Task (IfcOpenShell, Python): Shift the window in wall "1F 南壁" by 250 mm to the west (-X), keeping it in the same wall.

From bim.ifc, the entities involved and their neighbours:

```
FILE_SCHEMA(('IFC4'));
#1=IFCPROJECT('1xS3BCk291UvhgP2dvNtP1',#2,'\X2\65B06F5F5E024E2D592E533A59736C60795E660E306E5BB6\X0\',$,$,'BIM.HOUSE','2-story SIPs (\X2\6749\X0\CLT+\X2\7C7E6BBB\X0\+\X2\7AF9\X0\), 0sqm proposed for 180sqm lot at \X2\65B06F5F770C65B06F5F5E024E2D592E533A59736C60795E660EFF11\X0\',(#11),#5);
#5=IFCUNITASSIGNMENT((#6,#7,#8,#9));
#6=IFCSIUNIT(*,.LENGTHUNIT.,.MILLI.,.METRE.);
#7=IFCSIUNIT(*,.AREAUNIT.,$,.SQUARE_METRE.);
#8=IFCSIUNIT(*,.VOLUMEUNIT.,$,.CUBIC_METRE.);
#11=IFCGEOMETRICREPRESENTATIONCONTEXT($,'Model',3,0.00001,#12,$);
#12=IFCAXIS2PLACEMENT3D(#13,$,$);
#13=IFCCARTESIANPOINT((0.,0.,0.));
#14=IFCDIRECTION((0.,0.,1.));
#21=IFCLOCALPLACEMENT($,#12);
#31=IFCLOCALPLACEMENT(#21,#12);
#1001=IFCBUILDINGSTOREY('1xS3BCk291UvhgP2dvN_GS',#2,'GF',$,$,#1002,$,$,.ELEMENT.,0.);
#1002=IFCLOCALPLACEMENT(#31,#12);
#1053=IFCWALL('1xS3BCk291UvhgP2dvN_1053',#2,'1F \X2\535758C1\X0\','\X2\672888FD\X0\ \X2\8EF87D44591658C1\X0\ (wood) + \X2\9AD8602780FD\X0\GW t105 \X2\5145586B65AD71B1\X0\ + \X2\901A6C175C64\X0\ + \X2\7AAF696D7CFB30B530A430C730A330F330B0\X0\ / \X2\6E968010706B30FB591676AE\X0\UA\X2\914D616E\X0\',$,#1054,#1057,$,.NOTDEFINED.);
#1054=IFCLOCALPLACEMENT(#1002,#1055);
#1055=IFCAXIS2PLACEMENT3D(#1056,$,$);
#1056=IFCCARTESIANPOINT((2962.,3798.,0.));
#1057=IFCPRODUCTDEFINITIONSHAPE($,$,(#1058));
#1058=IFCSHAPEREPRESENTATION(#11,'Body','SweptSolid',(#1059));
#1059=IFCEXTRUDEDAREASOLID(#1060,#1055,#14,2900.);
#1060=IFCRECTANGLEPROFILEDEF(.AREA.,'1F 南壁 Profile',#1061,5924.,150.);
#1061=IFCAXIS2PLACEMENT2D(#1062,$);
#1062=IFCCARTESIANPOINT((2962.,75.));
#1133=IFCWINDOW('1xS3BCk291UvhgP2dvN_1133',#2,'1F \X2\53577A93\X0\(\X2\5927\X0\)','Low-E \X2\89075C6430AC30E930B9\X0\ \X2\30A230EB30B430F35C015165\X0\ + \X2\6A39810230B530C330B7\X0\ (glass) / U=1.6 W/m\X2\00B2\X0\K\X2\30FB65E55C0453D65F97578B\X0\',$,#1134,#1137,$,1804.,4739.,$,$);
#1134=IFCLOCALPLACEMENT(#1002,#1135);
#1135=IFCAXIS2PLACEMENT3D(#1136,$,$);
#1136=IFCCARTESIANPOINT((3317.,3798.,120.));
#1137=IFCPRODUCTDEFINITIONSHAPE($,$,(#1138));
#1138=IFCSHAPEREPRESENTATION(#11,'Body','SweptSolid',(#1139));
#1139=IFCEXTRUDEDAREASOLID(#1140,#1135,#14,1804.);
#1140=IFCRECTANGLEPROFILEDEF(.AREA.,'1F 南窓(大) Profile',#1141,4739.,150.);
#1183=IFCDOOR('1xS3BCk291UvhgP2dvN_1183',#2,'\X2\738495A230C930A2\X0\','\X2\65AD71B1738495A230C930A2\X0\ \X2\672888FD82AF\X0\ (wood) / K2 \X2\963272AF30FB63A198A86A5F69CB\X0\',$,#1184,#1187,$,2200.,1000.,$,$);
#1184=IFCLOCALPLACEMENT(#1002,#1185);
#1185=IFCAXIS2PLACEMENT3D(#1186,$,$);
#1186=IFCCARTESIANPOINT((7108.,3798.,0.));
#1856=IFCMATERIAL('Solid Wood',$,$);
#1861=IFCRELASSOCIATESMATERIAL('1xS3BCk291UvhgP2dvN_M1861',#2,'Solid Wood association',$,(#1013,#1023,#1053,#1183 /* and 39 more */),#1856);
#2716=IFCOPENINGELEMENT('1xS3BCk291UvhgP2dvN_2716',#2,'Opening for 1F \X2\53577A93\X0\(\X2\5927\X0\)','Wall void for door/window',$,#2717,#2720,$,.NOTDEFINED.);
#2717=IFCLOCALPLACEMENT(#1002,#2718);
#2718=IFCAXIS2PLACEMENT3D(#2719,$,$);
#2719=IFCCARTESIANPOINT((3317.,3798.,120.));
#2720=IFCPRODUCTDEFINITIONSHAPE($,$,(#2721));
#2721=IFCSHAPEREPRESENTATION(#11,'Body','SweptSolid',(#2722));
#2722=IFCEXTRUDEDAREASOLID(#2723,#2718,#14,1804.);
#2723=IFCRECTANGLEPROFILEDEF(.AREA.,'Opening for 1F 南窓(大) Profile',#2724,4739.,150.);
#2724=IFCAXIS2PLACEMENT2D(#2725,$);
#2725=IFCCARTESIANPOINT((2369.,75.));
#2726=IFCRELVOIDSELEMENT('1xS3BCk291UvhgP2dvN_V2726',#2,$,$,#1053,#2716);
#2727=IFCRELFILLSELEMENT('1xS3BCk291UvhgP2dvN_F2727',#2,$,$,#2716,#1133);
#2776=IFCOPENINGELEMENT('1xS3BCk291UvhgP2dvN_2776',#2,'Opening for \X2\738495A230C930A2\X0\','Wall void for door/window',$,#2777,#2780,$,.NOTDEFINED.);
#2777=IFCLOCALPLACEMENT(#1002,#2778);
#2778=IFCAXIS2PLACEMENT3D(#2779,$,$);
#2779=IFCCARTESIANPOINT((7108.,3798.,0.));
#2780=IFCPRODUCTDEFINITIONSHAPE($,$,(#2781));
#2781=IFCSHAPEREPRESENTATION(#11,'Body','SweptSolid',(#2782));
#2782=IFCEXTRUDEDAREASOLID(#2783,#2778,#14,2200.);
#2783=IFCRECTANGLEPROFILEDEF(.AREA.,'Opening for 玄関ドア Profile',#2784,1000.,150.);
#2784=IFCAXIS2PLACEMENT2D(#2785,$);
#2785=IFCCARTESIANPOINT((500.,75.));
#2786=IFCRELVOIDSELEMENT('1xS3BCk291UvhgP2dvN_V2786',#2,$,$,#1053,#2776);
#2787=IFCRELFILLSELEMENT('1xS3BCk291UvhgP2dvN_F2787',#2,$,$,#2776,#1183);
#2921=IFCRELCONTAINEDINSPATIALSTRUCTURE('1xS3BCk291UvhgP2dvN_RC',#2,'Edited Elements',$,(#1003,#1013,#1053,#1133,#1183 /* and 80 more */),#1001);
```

```python
import ifcopenshell
import ifcopenshell.api.geometry
import ifcopenshell.util.placement

model = ifcopenshell.open("bim.ifc")

window = model.by_guid("1xS3BCk291UvhgP2dvN_1133")
opening = window.FillsVoids[0].RelatingOpeningElement
wall = opening.VoidsElements[0].RelatingBuildingElement

wall_matrix = ifcopenshell.util.placement.get_local_placement(wall.ObjectPlacement)
shift = wall_matrix[:3, 0] * -250.0
before = ifcopenshell.util.placement.get_local_placement(window.ObjectPlacement)[:3, 3].copy()

# The window is not placed relative to its opening, so move both.
for product in (opening, window):
    matrix = ifcopenshell.util.placement.get_local_placement(product.ObjectPlacement)
    matrix[:3, 3] += shift
    ifcopenshell.api.geometry.edit_object_placement(model, product=product, matrix=matrix, is_si=False)

after = ifcopenshell.util.placement.get_local_placement(window.ObjectPlacement)[:3, 3]
print("window moved by", (after - before).round(3) + 0.0)

model.write("bim_rev.ifc")
```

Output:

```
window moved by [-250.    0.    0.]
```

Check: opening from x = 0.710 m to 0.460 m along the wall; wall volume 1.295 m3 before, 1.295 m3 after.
